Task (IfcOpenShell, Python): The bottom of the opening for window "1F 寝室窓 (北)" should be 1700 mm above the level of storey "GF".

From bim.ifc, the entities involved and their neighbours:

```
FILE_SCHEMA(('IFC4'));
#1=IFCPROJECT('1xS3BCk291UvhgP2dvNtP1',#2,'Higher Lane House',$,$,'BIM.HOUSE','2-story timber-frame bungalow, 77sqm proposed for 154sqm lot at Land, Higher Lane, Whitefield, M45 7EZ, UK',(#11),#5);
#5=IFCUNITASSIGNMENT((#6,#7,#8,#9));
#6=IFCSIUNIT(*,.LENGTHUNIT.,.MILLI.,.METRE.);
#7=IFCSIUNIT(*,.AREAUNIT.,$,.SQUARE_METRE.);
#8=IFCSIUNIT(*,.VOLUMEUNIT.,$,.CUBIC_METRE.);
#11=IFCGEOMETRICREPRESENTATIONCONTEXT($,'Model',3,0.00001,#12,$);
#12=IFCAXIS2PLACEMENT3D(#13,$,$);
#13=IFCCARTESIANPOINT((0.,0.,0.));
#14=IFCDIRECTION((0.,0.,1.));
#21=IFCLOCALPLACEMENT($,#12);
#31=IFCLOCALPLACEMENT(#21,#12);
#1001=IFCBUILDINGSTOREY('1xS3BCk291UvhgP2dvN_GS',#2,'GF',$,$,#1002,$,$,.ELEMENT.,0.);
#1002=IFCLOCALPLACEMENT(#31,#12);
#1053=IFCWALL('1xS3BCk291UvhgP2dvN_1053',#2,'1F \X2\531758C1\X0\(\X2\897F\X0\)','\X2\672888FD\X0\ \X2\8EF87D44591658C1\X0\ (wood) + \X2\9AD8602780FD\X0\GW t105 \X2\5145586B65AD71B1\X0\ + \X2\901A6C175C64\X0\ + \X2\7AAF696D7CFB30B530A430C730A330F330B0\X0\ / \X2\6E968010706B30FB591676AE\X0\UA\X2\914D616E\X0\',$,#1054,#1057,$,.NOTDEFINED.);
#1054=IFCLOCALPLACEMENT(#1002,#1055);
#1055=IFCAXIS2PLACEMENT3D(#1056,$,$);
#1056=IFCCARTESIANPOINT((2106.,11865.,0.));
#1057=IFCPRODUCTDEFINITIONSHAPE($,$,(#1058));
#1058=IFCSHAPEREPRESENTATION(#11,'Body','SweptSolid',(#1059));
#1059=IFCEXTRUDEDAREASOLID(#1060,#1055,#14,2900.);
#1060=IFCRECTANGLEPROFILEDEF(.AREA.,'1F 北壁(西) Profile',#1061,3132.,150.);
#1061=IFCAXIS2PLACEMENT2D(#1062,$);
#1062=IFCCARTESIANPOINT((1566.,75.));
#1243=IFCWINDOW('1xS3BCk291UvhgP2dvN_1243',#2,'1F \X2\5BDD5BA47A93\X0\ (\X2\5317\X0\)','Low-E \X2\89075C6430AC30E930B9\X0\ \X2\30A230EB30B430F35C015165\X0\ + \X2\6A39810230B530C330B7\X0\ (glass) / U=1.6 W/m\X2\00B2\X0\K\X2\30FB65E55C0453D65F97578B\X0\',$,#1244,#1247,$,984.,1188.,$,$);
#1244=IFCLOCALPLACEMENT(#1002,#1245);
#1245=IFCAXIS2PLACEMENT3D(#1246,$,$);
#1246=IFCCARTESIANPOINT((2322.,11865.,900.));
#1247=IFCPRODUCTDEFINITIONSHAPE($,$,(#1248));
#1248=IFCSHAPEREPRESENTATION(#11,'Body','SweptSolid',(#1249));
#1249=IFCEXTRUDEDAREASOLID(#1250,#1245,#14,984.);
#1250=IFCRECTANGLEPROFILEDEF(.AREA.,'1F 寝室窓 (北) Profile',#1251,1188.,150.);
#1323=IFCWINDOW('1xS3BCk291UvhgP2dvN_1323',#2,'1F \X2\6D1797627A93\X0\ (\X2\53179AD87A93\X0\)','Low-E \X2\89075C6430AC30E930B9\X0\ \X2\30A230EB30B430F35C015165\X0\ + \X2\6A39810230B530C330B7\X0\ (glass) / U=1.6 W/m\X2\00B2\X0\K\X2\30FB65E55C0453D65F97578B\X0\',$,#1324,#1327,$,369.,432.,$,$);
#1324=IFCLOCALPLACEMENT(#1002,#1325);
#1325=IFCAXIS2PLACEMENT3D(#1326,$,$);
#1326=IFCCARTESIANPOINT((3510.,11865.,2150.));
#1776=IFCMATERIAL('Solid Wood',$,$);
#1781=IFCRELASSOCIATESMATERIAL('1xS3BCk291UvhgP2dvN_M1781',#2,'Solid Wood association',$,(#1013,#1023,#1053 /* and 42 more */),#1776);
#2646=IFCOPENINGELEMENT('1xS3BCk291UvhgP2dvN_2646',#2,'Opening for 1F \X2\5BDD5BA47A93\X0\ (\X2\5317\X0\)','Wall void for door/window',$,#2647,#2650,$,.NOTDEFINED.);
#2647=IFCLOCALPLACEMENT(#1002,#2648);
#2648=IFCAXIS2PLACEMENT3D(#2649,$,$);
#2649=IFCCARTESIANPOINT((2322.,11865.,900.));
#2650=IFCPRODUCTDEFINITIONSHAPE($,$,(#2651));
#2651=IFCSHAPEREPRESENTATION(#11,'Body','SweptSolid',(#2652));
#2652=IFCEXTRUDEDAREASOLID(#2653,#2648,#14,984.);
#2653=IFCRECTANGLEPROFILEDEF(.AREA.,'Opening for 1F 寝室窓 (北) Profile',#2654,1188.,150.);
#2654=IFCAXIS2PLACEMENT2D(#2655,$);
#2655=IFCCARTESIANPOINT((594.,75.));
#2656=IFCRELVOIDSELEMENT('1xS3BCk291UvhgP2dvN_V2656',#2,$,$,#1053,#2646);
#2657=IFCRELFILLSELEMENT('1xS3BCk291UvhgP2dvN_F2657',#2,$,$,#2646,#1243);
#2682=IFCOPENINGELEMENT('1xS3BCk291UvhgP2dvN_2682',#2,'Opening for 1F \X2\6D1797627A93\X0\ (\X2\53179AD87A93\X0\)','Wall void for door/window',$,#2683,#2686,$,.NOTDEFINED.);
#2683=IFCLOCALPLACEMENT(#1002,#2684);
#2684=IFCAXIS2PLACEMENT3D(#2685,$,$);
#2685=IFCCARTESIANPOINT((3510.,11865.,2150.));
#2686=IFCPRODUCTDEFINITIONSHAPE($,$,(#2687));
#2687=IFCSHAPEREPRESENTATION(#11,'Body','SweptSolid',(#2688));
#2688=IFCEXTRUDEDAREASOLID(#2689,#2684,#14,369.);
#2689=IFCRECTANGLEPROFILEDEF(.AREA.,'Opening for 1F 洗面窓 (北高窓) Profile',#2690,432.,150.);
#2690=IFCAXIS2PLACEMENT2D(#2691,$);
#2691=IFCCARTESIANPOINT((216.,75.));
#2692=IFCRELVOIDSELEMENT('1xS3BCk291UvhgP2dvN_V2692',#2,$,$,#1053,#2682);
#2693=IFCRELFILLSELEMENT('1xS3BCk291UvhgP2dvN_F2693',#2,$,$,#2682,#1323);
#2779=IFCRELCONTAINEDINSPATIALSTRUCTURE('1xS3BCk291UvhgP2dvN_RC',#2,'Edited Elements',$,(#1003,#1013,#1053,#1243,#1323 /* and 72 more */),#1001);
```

```python
import numpy as np
import ifcopenshell
import ifcopenshell.api.geometry
import ifcopenshell.geom
import ifcopenshell.util.element
import ifcopenshell.util.placement
import ifcopenshell.util.shape
import ifcopenshell.util.unit

model = ifcopenshell.open("bim.ifc")
unit_scale = ifcopenshell.util.unit.calculate_unit_scale(model)

window = model.by_guid("1xS3BCk291UvhgP2dvN_1243")
opening = window.FillsVoids[0].RelatingOpeningElement
storey = ifcopenshell.util.element.get_container(window, ifc_class="IfcBuildingStorey")
level = ifcopenshell.util.placement.get_local_placement(storey.ObjectPlacement)[2, 3]

# The opening's origin need not be at the sill, so measure its lowest point.
shape = ifcopenshell.geom.create_shape(ifcopenshell.geom.settings(), opening)
bottom = ifcopenshell.util.shape.get_shape_bottom_elevation(shape, shape.geometry) / unit_scale
dz = level + 1.7 / unit_scale - bottom

shift = np.array([0.0, 0.0, dz])
# The window is not placed relative to its opening, so move both.
for product in (opening, window):
    matrix = ifcopenshell.util.placement.get_local_placement(product.ObjectPlacement)
    matrix[:3, 3] += shift
    ifcopenshell.api.geometry.edit_object_placement(model, product=product, matrix=matrix, is_si=False)

print(f"moved by {dz * unit_scale:+.3f} m")

model.write("bim_v2.ifc")
```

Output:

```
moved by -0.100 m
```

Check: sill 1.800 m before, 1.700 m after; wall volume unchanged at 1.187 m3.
